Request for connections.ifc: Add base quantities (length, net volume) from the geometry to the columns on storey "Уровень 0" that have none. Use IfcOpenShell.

First a look at what the model holds.

```python
import ifcopenshell
import ifcopenshell.util.element
import ifcopenshell.util.unit

model = ifcopenshell.open("connections.ifc")
print(model.schema)
for unit_type in ("LENGTHUNIT", "AREAUNIT", "VOLUMEUNIT"):
    print(unit_type, ifcopenshell.util.unit.calculate_unit_scale(model, unit_type))
storey = next(s for s in model.by_type("IfcBuildingStorey") if s.Name == "Уровень 0")
columns = [e for e in ifcopenshell.util.element.get_decomposition(storey) if e.is_a("IfcColumn")]
for e in sorted(columns, key=lambda e: e.id()):
    print(e.id(), e.is_a(), e.Name, list(ifcopenshell.util.element.get_psets(e, qtos_only=True)), sep=" | ")
```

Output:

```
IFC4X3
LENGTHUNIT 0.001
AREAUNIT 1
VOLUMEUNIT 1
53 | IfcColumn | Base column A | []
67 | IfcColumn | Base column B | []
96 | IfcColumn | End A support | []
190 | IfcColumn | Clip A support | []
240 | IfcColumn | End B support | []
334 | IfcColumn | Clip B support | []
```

```python
import ifcopenshell
import ifcopenshell.api.pset
import ifcopenshell.geom
import ifcopenshell.util.element
import ifcopenshell.util.shape
import ifcopenshell.util.unit

model = ifcopenshell.open("connections.ifc")
unit_scale = ifcopenshell.util.unit.calculate_unit_scale(model)
volume_scale = ifcopenshell.util.unit.calculate_unit_scale(model, "VOLUMEUNIT")
settings = ifcopenshell.geom.settings()

storey = next(s for s in model.by_type("IfcBuildingStorey") if s.Name == "Уровень 0")
columns = [e for e in ifcopenshell.util.element.get_decomposition(storey) if e.is_a("IfcColumn")]

for e in sorted(columns, key=lambda e: e.id()):
    if ifcopenshell.util.element.get_psets(e, qtos_only=True, should_inherit=False):
        continue
    # Geometry comes back in metres, in the element's own axes.
    shape = ifcopenshell.geom.create_shape(settings, e)
    values = {
        "Length": ifcopenshell.util.shape.get_z(shape.geometry) / unit_scale,
        "NetVolume": ifcopenshell.util.shape.get_volume(shape.geometry) / volume_scale,
    }
    qto = ifcopenshell.api.pset.add_qto(model, product=e, name="Qto_ColumnBaseQuantities")
    ifcopenshell.api.pset.edit_qto(model, qto=qto, properties=values)
    print(e.id(), {k: round(v, 3) for k, v in values.items()})

model.write("connections_rev.ifc")
```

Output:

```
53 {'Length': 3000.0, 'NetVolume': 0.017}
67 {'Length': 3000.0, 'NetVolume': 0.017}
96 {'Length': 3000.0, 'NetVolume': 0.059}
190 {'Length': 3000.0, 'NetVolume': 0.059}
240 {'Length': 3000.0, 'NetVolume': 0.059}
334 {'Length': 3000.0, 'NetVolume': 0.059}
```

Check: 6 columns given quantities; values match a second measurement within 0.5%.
